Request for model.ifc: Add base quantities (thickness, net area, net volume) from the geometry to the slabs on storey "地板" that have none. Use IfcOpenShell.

First a look at what the model holds.

```python
import ifcopenshell
import ifcopenshell.util.element
import ifcopenshell.util.unit

model = ifcopenshell.open("model.ifc")
print(model.schema)
for unit_type in ("LENGTHUNIT", "AREAUNIT", "VOLUMEUNIT"):
    print(unit_type, ifcopenshell.util.unit.calculate_unit_scale(model, unit_type))
storey = next(s for s in model.by_type("IfcBuildingStorey") if s.Name == "地板")
slabs = [e for e in ifcopenshell.util.element.get_decomposition(storey) if e.is_a("IfcSlab")]
for e in sorted(slabs, key=lambda e: e.id()):
    print(e.id(), e.is_a(), e.Name, list(ifcopenshell.util.element.get_psets(e, qtos_only=True)), sep=" | ")
```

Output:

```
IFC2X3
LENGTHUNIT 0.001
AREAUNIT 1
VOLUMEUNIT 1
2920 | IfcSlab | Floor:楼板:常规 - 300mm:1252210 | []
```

```python
import ifcopenshell
import ifcopenshell.api.pset
import ifcopenshell.geom
import ifcopenshell.util.element
import ifcopenshell.util.shape
import ifcopenshell.util.unit

model = ifcopenshell.open("model.ifc")
unit_scale = ifcopenshell.util.unit.calculate_unit_scale(model)
area_scale = ifcopenshell.util.unit.calculate_unit_scale(model, "AREAUNIT")
volume_scale = ifcopenshell.util.unit.calculate_unit_scale(model, "VOLUMEUNIT")
settings = ifcopenshell.geom.settings()

storey = next(s for s in model.by_type("IfcBuildingStorey") if s.Name == "地板")
slabs = [e for e in ifcopenshell.util.element.get_decomposition(storey) if e.is_a("IfcSlab")]

for e in sorted(slabs, key=lambda e: e.id()):
    if ifcopenshell.util.element.get_psets(e, qtos_only=True, should_inherit=False):
        continue
    # Geometry comes back in metres, in the element's own axes.
    shape = ifcopenshell.geom.create_shape(settings, e)
    values = {
        "Width": ifcopenshell.util.shape.get_z(shape.geometry) / unit_scale,
        "NetArea": ifcopenshell.util.shape.get_footprint_area(shape.geometry) / area_scale,
        "NetVolume": ifcopenshell.util.shape.get_volume(shape.geometry) / volume_scale,
    }
    qto = ifcopenshell.api.pset.add_qto(model, product=e, name="BaseQuantities")
    ifcopenshell.api.pset.edit_qto(model, qto=qto, properties=values)
    print(e.id(), {k: round(v, 3) for k, v in values.items()})

model.write("model_v2.ifc")
```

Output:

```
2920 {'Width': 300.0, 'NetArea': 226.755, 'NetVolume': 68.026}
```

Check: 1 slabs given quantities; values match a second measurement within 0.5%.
